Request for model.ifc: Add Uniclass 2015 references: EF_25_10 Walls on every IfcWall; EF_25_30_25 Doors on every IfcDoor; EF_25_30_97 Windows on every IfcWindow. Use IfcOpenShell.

First a look at what the model holds.

```python
import ifcopenshell

model = ifcopenshell.open("model.ifc")
print(model.schema)
print("classifications:", [c.Name for c in model.by_type("IfcClassification")])
for ifc_class in ("IfcDoor", "IfcRoof", "IfcStair", "IfcWall", "IfcWindow"):
    print(ifc_class, len(model.by_type(ifc_class)))
```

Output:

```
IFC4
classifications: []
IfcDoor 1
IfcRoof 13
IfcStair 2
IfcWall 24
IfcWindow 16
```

```python
import ifcopenshell
import ifcopenshell.api.classification

model = ifcopenshell.open("model.ifc")

system = ifcopenshell.api.classification.add_classification(model, classification="Uniclass 2015")

codes = {
    "IfcWall": ("EF_25_10", "Walls"),
    "IfcDoor": ("EF_25_30_25", "Doors"),
    "IfcWindow": ("EF_25_30_97", "Windows"),
}
for ifc_class, (code, name) in codes.items():
    products = model.by_type(ifc_class)
    ifcopenshell.api.classification.add_reference(
        model, products=products, classification=system, identification=code, name=name
    )
    print(code, len(products))

model.write("model_updated.ifc")
```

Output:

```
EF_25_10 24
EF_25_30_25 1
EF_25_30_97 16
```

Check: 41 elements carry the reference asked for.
